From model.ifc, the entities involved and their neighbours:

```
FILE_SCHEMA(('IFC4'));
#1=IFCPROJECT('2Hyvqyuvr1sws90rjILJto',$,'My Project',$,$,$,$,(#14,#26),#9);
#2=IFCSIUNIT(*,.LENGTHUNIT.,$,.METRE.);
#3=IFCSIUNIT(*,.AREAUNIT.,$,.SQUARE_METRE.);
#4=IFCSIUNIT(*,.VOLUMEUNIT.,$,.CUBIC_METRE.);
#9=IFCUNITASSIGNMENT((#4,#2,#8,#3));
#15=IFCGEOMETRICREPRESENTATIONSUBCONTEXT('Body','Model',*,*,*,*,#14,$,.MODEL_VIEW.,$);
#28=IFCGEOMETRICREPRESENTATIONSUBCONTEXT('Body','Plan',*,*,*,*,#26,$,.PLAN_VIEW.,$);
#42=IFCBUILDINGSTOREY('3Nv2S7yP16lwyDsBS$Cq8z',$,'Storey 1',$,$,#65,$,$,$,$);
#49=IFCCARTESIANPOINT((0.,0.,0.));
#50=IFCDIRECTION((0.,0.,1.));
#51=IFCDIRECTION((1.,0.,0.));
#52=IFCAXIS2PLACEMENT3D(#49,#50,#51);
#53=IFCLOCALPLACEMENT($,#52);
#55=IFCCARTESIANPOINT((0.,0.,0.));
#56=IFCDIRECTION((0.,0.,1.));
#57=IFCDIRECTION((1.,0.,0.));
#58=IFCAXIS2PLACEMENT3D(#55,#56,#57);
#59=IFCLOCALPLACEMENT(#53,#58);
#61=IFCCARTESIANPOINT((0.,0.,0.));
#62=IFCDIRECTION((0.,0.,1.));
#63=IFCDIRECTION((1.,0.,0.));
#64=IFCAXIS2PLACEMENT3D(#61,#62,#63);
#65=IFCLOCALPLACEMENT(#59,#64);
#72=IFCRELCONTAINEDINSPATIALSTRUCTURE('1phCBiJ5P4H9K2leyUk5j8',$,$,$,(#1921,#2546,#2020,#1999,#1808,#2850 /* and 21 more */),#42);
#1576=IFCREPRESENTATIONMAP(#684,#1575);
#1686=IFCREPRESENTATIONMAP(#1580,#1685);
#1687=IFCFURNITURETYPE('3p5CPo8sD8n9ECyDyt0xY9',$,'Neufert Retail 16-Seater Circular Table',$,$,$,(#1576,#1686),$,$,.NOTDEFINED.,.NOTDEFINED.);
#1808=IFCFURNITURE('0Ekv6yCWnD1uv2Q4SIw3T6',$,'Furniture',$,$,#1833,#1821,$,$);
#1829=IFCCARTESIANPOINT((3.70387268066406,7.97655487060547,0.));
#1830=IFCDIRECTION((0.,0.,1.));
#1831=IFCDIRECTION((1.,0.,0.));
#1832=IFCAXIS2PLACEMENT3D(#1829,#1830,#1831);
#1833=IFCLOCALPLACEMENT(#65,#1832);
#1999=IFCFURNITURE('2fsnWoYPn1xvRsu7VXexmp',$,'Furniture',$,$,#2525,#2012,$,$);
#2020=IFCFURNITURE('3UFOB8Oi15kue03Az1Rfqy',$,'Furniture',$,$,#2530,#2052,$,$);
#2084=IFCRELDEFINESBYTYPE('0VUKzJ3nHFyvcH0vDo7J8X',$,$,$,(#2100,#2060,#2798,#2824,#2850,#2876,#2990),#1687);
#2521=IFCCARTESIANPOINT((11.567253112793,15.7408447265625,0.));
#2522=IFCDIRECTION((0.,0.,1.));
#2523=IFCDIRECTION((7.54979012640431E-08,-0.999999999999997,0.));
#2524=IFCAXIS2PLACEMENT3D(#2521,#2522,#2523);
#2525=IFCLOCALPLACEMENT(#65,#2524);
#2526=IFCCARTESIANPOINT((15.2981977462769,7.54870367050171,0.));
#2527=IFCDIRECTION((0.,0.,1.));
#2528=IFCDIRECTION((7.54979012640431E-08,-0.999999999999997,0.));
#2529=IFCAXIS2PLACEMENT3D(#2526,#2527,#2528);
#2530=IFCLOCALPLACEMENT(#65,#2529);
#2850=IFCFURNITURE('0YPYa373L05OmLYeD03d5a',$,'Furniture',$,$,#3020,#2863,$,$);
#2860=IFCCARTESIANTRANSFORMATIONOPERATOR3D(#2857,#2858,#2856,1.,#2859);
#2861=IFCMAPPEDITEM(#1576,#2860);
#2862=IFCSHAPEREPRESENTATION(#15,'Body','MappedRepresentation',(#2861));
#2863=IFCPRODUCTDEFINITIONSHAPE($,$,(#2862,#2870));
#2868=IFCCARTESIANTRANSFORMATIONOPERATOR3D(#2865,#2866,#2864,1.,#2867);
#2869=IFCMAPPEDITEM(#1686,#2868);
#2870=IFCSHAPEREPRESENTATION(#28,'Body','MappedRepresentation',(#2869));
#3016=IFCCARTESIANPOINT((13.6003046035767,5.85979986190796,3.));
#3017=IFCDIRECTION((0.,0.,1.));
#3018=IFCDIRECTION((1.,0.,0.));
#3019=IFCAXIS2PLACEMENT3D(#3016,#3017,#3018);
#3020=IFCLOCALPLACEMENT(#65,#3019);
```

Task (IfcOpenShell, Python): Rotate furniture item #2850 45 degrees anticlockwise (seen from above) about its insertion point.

```python
import ifcopenshell
import ifcopenshell.api.geometry
import ifcopenshell.util.placement

model = ifcopenshell.open("model.ifc")

item = model.by_id(2850)
matrix = ifcopenshell.util.placement.get_local_placement(item.ObjectPlacement)
matrix = matrix @ ifcopenshell.util.placement.rotation(45, "Z")
ifcopenshell.api.geometry.edit_object_placement(model, product=item, matrix=matrix, is_si=False)

print(ifcopenshell.util.placement.get_local_placement(item.ObjectPlacement).round(3) + 0.0)

model.write("model_rev.ifc")
```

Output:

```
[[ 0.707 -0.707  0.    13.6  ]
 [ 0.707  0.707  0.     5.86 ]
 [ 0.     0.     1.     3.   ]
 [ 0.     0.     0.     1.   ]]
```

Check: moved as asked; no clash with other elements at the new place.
